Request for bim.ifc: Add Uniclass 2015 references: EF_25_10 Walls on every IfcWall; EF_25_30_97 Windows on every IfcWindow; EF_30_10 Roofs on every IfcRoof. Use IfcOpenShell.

First a look at what the model holds.

```python
import ifcopenshell

model = ifcopenshell.open("bim.ifc")
print(model.schema)
print("classifications:", [c.Name for c in model.by_type("IfcClassification")])
for ifc_class in ("IfcDoor", "IfcRoof", "IfcStair", "IfcWall", "IfcWindow"):
    print(ifc_class, len(model.by_type(ifc_class)))
```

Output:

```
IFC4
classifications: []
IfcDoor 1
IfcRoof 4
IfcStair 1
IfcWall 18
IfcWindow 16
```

```python
import ifcopenshell
import ifcopenshell.api.classification

model = ifcopenshell.open("bim.ifc")

system = ifcopenshell.api.classification.add_classification(model, classification="Uniclass 2015")

codes = {
    "IfcWall": ("EF_25_10", "Walls"),
    "IfcWindow": ("EF_25_30_97", "Windows"),
    "IfcRoof": ("EF_30_10", "Roofs"),
}
for ifc_class, (code, name) in codes.items():
    products = model.by_type(ifc_class)
    ifcopenshell.api.classification.add_reference(
        model, products=products, classification=system, identification=code, name=name
    )
    print(code, len(products))

model.write("bim_v2.ifc")
```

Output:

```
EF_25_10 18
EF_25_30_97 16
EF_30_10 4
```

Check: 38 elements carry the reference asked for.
